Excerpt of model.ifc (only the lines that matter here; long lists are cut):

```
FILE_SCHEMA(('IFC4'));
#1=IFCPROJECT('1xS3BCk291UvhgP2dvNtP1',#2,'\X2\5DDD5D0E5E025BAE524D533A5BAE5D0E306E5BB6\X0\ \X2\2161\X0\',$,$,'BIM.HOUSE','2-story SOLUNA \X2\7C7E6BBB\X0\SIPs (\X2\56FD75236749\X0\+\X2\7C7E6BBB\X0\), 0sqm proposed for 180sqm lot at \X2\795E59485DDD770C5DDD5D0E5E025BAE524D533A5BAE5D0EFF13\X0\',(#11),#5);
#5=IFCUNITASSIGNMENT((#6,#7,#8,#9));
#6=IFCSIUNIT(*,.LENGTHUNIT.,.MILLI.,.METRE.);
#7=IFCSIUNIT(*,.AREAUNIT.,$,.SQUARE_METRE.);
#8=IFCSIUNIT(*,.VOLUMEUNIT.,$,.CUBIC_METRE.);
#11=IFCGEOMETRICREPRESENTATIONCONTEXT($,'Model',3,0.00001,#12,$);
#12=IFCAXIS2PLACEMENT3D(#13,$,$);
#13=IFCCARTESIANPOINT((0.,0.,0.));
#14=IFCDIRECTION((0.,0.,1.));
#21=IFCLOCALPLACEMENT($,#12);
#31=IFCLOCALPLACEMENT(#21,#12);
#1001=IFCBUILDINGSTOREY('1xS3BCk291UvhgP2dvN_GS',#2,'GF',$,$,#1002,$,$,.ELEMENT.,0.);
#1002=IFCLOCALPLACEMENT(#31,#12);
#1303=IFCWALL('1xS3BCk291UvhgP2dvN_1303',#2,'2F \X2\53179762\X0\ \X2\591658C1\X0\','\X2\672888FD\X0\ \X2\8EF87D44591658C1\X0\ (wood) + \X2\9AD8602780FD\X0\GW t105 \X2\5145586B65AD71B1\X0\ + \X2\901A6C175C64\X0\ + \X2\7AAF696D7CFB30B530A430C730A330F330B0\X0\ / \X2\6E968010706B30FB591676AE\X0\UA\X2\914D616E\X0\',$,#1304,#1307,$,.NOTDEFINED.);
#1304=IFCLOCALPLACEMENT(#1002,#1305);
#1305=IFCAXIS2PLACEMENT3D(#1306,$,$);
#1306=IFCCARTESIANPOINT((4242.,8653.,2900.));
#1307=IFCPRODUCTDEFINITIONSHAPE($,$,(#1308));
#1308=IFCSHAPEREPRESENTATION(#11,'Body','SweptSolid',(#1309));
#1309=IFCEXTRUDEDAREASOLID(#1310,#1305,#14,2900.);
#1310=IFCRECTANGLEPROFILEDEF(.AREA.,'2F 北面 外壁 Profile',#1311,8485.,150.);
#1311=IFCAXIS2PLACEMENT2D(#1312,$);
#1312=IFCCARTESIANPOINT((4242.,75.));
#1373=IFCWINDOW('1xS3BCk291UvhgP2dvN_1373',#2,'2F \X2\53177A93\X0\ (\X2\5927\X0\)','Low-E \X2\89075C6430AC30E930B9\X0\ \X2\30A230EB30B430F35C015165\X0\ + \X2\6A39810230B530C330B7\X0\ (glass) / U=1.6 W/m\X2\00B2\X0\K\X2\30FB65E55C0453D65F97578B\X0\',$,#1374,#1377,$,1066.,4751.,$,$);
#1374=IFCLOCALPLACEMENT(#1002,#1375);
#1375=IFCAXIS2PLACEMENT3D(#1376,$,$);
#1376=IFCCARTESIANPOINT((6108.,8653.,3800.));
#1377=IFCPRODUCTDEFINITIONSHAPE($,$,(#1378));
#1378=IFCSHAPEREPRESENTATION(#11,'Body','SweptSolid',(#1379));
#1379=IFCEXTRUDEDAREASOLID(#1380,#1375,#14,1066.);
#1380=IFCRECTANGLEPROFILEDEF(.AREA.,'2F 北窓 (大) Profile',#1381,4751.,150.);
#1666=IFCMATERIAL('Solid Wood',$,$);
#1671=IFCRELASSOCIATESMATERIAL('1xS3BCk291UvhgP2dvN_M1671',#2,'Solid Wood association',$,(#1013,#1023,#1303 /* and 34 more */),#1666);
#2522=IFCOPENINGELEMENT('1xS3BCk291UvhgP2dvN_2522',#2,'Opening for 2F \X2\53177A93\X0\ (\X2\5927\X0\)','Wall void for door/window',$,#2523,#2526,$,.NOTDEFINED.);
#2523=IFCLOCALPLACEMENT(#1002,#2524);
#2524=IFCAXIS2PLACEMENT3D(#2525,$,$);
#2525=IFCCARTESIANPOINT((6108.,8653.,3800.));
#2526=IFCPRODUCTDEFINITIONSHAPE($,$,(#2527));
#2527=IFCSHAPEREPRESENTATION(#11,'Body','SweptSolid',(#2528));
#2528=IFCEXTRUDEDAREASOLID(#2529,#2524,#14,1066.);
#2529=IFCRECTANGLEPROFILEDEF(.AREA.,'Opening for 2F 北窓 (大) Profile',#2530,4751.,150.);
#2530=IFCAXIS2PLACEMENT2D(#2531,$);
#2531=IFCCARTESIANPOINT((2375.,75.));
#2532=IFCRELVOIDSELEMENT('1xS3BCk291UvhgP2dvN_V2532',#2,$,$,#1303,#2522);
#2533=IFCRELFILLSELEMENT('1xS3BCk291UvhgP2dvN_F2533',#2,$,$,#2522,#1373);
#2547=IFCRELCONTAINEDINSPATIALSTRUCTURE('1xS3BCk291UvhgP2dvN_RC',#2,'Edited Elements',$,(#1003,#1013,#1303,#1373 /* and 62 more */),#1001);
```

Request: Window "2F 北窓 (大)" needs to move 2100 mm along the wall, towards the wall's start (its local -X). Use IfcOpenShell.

```python
import ifcopenshell
import ifcopenshell.api.geometry
import ifcopenshell.util.placement
import ifcopenshell.util.unit

model = ifcopenshell.open("model.ifc")
unit_scale = ifcopenshell.util.unit.calculate_unit_scale(model)

window = model.by_guid("1xS3BCk291UvhgP2dvN_1373")
opening = window.FillsVoids[0].RelatingOpeningElement
wall = opening.VoidsElements[0].RelatingBuildingElement

wall_matrix = ifcopenshell.util.placement.get_local_placement(wall.ObjectPlacement)
shift = wall_matrix[:3, 0] * -2.1 / unit_scale
before = ifcopenshell.util.placement.get_local_placement(window.ObjectPlacement)[:3, 3].copy()

# The window is not placed relative to its opening, so move both.
for product in (opening, window):
    matrix = ifcopenshell.util.placement.get_local_placement(product.ObjectPlacement)
    matrix[:3, 3] += shift
    ifcopenshell.api.geometry.edit_object_placement(model, product=product, matrix=matrix, is_si=False)

after = ifcopenshell.util.placement.get_local_placement(window.ObjectPlacement)[:3, 3]
print("window moved by", (after - before).round(3) + 0.0)

model.write("model_edited.ifc")
```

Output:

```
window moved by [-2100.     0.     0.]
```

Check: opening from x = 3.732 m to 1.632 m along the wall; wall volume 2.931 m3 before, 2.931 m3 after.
